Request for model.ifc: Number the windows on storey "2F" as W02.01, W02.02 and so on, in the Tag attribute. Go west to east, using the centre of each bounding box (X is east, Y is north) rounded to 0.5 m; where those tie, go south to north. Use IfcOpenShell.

First a look at what the model holds.

```python
import ifcopenshell
import ifcopenshell.util.element
import ifcopenshell.util.placement

model = ifcopenshell.open("model.ifc")
print(model.schema)
storey = next(s for s in model.by_type("IfcBuildingStorey") if s.Name == "2F")
windows = [e for e in ifcopenshell.util.element.get_decomposition(storey) if e.is_a("IfcWindow")]
for e in sorted(windows, key=lambda e: e.id()):
    origin = ifcopenshell.util.placement.get_local_placement(e.ObjectPlacement)[:3, 3]
    print(e.id(), e.Tag, e.Name, origin.round(2) + 0.0, sep=" | ")
```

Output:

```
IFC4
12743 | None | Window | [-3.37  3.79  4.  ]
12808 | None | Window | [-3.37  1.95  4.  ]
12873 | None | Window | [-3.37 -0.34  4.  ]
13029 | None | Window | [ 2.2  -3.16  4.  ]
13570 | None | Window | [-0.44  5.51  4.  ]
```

```python
import ifcopenshell
import ifcopenshell.geom
import ifcopenshell.util.element
import ifcopenshell.util.shape

model = ifcopenshell.open("model.ifc")
settings = ifcopenshell.geom.settings()
settings.set("use-world-coords", True)


def centre(element):
    shape = ifcopenshell.geom.create_shape(settings, element)
    return ifcopenshell.util.shape.get_bbox_centroid(shape.geometry)


storey = next(s for s in model.by_type("IfcBuildingStorey") if s.Name == "2F")
windows = [e for e in ifcopenshell.util.element.get_decomposition(storey) if e.is_a("IfcWindow")]

# Insertion points can sit at a corner or the storey origin, so sort by the geometry (in metres).
centres = {e: centre(e) for e in windows}
windows.sort(key=lambda e: (round(centres[e][0] / 0.5), centres[e][1]))

for i, e in enumerate(windows, start=1):
    number = f"W02.{i:02d}"
    e.Tag = number
    print(e.id(), number)

model.write("model-out.ifc")
```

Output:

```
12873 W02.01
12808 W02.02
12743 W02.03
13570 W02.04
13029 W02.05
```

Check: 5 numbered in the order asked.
